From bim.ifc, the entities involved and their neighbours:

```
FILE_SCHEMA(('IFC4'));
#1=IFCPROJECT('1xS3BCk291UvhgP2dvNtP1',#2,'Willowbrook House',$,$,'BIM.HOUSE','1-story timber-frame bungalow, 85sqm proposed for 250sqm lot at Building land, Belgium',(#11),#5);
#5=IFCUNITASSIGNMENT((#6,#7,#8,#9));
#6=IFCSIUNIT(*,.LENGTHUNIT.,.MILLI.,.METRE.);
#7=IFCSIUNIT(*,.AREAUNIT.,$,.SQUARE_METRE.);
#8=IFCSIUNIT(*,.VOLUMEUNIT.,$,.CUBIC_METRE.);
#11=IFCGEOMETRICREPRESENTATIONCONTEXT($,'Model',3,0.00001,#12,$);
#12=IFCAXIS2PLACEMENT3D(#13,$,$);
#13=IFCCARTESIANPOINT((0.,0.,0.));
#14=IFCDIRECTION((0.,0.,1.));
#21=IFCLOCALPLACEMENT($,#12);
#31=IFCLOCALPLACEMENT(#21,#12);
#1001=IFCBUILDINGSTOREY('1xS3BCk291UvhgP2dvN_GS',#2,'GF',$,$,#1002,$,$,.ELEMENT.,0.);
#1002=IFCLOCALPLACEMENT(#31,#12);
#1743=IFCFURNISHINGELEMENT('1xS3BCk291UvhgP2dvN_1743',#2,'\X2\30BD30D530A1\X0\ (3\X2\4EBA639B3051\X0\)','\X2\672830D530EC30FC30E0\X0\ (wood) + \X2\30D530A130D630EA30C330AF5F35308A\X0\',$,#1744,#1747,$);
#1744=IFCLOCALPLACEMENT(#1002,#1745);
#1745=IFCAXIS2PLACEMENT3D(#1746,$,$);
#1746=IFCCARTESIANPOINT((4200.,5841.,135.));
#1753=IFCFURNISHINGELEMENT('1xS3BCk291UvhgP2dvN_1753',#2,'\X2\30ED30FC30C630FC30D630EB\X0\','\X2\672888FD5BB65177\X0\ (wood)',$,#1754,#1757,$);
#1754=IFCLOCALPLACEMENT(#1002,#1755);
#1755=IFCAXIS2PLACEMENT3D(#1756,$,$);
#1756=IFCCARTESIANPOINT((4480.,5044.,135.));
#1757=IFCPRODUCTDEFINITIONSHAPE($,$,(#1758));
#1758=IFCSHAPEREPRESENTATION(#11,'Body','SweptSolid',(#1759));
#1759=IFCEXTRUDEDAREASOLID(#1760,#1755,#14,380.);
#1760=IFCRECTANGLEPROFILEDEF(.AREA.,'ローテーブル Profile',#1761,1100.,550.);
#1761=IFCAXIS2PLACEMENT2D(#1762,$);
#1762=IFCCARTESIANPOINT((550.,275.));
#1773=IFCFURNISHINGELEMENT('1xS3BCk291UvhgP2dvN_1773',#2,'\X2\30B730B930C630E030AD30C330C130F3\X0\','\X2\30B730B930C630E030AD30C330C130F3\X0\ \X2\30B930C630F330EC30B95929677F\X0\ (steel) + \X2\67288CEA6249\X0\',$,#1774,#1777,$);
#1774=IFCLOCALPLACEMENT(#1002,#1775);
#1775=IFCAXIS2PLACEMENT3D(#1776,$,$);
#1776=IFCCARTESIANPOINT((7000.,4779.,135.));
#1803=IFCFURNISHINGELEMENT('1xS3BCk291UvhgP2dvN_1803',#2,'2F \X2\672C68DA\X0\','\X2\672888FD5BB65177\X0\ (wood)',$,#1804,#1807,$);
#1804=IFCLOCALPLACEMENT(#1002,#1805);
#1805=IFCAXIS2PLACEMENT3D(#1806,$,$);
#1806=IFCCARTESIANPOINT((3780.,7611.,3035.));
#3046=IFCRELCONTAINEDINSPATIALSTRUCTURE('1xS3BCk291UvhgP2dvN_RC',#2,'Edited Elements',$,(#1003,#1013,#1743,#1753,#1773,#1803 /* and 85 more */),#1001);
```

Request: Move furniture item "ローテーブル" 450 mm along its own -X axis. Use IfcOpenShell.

```python
import ifcopenshell
import ifcopenshell.api.geometry
import ifcopenshell.util.placement
import ifcopenshell.util.unit

model = ifcopenshell.open("bim.ifc")
unit_scale = ifcopenshell.util.unit.calculate_unit_scale(model)

item = model.by_id(1753)
matrix = ifcopenshell.util.placement.get_local_placement(item.ObjectPlacement)
matrix[:3, 3] -= matrix[:3, 0] * 0.45 / unit_scale
ifcopenshell.api.geometry.edit_object_placement(model, product=item, matrix=matrix, is_si=False)

print(ifcopenshell.util.placement.get_local_placement(item.ObjectPlacement).round(3) + 0.0)

model.write("bim_v2.ifc")
```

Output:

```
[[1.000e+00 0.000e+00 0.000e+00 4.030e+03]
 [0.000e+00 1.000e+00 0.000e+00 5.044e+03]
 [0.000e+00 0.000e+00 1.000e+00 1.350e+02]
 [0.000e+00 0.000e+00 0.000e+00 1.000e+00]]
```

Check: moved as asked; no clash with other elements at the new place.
